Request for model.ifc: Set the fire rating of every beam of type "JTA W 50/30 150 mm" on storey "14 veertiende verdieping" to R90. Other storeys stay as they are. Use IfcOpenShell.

First a look at what the model holds.

```python
import ifcopenshell
import ifcopenshell.util.element

model = ifcopenshell.open("model.ifc")
print(model.schema)
storey = next(s for s in model.by_type("IfcBuildingStorey") if s.Name == "14 veertiende verdieping")
beams = [e for e in ifcopenshell.util.element.get_decomposition(storey) if e.is_a("IfcBeam")]
seen = {}
for e in beams:
    element_type = ifcopenshell.util.element.get_type(e)
    key = (element_type.Name if element_type != e and element_type else None, ifcopenshell.util.element.get_pset(e, "Pset_BeamCommon", "FireRating"))
    seen[key] = seen.get(key, 0) + 1
for (name, value), count in sorted(seen.items(), key=str):
    print(count, "x", name, "|", value)
```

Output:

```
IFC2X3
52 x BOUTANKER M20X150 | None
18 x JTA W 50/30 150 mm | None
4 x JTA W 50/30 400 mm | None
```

```python
import ifcopenshell
import ifcopenshell.api.pset
import ifcopenshell.util.element

model = ifcopenshell.open("model.ifc")

storey = next(s for s in model.by_type("IfcBuildingStorey") if s.Name == "14 veertiende verdieping")
beams = [e for e in ifcopenshell.util.element.get_decomposition(storey) if e.is_a("IfcBeam")]

count = 0
for e in beams:
    element_type = ifcopenshell.util.element.get_type(e)
    if element_type in (None, e) or element_type.Name != "JTA W 50/30 150 mm":
        continue
    # add_pset returns the element's existing set when there is one.
    pset = ifcopenshell.api.pset.add_pset(model, product=e, name="Pset_BeamCommon")
    ifcopenshell.api.pset.edit_pset(model, pset=pset, properties={"FireRating": "R90"})
    count += 1

print(count, "beams updated")

model.write("model_edited.ifc")
```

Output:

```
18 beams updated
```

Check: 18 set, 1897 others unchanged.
